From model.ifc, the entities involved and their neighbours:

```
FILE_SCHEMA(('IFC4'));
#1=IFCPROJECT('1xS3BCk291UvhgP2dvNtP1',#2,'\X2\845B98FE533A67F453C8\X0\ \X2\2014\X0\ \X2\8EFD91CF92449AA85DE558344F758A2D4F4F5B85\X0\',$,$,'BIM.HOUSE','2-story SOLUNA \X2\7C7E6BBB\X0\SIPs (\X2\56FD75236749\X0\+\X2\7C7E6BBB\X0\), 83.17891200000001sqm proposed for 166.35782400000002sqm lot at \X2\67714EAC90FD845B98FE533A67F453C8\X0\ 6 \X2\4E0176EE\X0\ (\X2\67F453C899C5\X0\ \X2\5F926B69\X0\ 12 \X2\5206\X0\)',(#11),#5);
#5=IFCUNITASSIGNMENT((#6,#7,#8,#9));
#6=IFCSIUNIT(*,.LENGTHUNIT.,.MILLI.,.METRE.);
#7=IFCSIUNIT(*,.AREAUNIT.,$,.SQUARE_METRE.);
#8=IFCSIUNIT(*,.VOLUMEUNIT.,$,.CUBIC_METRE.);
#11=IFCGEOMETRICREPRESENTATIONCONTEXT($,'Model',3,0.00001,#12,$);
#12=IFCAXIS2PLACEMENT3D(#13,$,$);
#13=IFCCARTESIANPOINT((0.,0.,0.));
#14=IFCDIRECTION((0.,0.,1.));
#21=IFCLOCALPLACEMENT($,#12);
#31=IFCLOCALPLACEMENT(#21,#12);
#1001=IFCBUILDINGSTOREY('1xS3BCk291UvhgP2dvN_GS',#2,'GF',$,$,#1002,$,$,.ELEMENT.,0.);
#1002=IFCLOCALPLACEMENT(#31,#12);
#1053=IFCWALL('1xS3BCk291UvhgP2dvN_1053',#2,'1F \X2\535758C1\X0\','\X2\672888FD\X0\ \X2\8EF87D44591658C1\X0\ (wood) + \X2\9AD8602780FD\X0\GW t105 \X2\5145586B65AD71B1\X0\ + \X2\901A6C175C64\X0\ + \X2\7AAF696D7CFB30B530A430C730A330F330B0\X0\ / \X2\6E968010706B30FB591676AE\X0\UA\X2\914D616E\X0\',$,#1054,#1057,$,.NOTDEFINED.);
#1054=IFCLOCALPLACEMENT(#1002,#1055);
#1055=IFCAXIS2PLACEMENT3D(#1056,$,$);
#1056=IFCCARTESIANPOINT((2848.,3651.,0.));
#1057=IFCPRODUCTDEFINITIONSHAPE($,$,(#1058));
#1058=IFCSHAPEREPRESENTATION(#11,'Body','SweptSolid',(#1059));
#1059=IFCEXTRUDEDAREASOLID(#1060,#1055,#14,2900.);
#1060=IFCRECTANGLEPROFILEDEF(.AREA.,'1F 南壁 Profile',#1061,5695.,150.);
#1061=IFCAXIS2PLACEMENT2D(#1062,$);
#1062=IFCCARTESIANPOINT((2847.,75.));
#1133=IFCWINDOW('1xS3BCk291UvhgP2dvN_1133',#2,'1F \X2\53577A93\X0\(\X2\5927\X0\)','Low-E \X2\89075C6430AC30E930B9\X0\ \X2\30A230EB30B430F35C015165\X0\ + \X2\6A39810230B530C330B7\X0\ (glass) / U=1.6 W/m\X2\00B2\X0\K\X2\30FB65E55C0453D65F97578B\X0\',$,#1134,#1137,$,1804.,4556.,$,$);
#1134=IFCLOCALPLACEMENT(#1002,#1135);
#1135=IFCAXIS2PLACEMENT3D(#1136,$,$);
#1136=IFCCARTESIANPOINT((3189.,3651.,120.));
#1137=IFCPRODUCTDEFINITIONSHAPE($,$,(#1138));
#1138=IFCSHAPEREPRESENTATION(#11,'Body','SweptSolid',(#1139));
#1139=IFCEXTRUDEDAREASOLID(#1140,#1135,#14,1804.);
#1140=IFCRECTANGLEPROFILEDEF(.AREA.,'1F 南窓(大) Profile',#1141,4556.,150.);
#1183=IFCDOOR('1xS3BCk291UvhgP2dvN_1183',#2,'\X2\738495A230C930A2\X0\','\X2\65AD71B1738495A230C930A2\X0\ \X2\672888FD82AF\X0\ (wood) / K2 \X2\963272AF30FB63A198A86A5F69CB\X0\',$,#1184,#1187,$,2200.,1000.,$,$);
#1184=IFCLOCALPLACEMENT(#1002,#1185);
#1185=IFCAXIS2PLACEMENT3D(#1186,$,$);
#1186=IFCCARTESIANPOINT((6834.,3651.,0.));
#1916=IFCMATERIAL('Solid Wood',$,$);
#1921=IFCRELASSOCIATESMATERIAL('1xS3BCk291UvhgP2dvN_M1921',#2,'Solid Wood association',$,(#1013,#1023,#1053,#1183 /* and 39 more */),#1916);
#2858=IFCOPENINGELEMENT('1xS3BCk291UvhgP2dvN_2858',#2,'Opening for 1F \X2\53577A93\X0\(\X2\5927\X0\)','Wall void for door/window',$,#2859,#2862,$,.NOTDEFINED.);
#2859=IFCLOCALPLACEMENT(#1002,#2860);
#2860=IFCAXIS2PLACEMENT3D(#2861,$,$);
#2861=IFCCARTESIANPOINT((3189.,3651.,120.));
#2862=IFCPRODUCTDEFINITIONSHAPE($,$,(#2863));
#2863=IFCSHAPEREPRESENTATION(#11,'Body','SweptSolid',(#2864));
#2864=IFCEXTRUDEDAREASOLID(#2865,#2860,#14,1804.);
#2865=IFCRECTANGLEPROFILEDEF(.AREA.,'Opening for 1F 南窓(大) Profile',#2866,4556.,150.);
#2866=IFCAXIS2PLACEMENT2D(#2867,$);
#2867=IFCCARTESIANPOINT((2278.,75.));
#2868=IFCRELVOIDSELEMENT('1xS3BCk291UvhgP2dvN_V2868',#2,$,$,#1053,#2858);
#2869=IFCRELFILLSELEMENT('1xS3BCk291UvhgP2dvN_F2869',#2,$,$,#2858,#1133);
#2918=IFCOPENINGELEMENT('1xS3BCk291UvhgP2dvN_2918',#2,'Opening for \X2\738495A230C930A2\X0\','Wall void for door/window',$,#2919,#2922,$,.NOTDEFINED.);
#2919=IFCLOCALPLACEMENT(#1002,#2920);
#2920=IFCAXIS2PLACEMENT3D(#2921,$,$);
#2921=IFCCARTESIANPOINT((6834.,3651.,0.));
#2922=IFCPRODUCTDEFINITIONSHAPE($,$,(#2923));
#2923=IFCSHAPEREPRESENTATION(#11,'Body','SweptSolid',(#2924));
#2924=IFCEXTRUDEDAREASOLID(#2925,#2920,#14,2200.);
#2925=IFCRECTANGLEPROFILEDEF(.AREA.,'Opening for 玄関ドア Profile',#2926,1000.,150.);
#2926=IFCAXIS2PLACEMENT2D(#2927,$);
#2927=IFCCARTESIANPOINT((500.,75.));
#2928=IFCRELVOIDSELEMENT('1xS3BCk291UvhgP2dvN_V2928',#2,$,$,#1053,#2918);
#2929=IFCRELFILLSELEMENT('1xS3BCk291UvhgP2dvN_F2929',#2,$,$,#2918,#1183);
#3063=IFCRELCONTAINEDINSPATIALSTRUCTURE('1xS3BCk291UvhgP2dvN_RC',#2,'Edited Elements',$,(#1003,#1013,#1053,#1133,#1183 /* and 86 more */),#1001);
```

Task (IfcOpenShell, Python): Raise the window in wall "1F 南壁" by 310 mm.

```python
import numpy as np
import ifcopenshell
import ifcopenshell.api.geometry
import ifcopenshell.util.placement
import ifcopenshell.util.unit

model = ifcopenshell.open("model.ifc")
unit_scale = ifcopenshell.util.unit.calculate_unit_scale(model)

window = model.by_guid("1xS3BCk291UvhgP2dvN_1133")
opening = window.FillsVoids[0].RelatingOpeningElement
dz = 0.31 / unit_scale

shift = np.array([0.0, 0.0, dz])
# The window is not placed relative to its opening, so move both.
for product in (opening, window):
    matrix = ifcopenshell.util.placement.get_local_placement(product.ObjectPlacement)
    matrix[:3, 3] += shift
    ifcopenshell.api.geometry.edit_object_placement(model, product=product, matrix=matrix, is_si=False)

print(f"moved by {dz * unit_scale:+.3f} m")

model.write("model-out.ifc")
```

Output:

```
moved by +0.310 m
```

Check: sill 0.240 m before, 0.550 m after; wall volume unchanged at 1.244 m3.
